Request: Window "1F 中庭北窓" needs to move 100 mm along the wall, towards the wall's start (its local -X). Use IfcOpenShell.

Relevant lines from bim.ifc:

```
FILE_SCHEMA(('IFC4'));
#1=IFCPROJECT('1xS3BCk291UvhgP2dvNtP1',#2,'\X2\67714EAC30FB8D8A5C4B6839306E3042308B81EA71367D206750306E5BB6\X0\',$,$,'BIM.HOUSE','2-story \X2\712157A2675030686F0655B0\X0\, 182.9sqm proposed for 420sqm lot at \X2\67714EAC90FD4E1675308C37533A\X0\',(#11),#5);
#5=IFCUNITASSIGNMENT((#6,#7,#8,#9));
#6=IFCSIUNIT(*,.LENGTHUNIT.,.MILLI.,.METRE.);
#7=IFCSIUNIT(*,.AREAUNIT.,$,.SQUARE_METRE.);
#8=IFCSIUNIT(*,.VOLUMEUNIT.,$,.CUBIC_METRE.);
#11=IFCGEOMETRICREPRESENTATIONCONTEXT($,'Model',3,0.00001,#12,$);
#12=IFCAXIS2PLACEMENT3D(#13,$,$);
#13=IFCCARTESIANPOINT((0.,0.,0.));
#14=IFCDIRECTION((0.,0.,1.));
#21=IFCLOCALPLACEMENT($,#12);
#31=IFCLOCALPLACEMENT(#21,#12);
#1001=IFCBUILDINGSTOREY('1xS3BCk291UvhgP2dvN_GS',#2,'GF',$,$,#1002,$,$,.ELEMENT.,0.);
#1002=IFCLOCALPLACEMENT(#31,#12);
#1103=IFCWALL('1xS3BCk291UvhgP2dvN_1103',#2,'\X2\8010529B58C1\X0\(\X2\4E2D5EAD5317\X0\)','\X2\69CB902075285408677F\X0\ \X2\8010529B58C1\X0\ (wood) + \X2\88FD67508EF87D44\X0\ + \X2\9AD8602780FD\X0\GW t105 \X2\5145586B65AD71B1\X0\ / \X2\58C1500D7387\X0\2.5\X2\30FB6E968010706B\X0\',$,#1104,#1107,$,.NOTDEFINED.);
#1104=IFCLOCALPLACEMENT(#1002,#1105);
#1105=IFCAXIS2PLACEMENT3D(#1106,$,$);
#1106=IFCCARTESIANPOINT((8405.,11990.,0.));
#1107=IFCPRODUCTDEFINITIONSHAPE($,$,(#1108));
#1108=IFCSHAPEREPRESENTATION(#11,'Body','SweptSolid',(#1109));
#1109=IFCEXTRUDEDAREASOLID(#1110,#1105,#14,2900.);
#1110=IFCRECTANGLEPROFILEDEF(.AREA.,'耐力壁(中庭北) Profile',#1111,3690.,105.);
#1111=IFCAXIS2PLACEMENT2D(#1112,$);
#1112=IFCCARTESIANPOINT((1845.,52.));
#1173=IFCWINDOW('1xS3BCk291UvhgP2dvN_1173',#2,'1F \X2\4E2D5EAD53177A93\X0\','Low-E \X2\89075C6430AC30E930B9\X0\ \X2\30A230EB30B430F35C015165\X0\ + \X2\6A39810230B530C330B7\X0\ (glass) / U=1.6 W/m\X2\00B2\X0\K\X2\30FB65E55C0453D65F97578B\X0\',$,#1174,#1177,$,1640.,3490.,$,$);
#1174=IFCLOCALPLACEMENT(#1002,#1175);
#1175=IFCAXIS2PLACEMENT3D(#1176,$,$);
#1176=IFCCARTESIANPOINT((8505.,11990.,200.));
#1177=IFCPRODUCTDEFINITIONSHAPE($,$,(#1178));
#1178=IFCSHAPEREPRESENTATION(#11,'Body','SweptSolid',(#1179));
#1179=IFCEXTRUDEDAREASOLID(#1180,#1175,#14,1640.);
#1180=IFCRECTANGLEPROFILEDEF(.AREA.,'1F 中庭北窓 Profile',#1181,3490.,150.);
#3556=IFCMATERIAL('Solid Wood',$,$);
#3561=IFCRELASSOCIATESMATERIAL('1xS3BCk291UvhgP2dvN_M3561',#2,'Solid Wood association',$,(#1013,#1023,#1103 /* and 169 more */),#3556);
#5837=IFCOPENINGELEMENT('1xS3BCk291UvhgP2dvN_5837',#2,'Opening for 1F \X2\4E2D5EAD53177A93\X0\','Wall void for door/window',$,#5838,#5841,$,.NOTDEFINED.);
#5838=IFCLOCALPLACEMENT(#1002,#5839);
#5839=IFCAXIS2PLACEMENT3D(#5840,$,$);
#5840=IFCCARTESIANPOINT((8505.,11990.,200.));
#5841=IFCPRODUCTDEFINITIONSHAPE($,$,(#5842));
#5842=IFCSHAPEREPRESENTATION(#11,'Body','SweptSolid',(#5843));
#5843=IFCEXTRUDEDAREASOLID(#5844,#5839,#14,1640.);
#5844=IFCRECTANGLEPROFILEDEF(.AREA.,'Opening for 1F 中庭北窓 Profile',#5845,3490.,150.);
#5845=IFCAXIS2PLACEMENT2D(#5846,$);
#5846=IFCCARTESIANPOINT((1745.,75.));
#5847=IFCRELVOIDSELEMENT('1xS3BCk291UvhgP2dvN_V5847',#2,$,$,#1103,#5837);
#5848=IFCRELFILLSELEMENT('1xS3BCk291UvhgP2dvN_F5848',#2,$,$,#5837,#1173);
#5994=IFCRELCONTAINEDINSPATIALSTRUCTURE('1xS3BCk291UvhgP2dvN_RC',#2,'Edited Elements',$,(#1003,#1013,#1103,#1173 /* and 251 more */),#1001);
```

```python
import ifcopenshell
import ifcopenshell.api.geometry
import ifcopenshell.util.placement

model = ifcopenshell.open("bim.ifc")

window = model.by_id(1173)
opening = window.FillsVoids[0].RelatingOpeningElement
wall = opening.VoidsElements[0].RelatingBuildingElement

wall_matrix = ifcopenshell.util.placement.get_local_placement(wall.ObjectPlacement)
shift = wall_matrix[:3, 0] * -100.0
before = ifcopenshell.util.placement.get_local_placement(window.ObjectPlacement)[:3, 3].copy()

# The window is not placed relative to its opening, so move both.
for product in (opening, window):
    matrix = ifcopenshell.util.placement.get_local_placement(product.ObjectPlacement)
    matrix[:3, 3] += shift
    ifcopenshell.api.geometry.edit_object_placement(model, product=product, matrix=matrix, is_si=False)

after = ifcopenshell.util.placement.get_local_placement(window.ObjectPlacement)[:3, 3]
print("window moved by", (after - before).round(3) + 0.0)

model.write("bim_updated.ifc")
```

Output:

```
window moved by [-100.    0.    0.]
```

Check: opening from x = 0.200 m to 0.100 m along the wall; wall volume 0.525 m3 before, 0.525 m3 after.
